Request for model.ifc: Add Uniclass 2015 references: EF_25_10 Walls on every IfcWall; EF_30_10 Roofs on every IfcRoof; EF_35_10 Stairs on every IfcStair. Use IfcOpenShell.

First a look at what the model holds.

```python
import ifcopenshell

model = ifcopenshell.open("model.ifc")
print(model.schema)
print("classifications:", [c.Name for c in model.by_type("IfcClassification")])
for ifc_class in ("IfcDoor", "IfcRoof", "IfcStair", "IfcWall", "IfcWindow"):
    print(ifc_class, len(model.by_type(ifc_class)))
```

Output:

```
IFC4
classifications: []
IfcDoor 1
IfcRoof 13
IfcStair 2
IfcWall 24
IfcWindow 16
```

```python
import ifcopenshell
import ifcopenshell.api.classification

model = ifcopenshell.open("model.ifc")

system = ifcopenshell.api.classification.add_classification(model, classification="Uniclass 2015")

codes = {
    "IfcWall": ("EF_25_10", "Walls"),
    "IfcRoof": ("EF_30_10", "Roofs"),
    "IfcStair": ("EF_35_10", "Stairs"),
}
for ifc_class, (code, name) in codes.items():
    products = model.by_type(ifc_class)
    ifcopenshell.api.classification.add_reference(
        model, products=products, classification=system, identification=code, name=name
    )
    print(code, len(products))

model.write("model_v2.ifc")
```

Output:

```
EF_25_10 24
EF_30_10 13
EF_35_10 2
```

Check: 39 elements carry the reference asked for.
